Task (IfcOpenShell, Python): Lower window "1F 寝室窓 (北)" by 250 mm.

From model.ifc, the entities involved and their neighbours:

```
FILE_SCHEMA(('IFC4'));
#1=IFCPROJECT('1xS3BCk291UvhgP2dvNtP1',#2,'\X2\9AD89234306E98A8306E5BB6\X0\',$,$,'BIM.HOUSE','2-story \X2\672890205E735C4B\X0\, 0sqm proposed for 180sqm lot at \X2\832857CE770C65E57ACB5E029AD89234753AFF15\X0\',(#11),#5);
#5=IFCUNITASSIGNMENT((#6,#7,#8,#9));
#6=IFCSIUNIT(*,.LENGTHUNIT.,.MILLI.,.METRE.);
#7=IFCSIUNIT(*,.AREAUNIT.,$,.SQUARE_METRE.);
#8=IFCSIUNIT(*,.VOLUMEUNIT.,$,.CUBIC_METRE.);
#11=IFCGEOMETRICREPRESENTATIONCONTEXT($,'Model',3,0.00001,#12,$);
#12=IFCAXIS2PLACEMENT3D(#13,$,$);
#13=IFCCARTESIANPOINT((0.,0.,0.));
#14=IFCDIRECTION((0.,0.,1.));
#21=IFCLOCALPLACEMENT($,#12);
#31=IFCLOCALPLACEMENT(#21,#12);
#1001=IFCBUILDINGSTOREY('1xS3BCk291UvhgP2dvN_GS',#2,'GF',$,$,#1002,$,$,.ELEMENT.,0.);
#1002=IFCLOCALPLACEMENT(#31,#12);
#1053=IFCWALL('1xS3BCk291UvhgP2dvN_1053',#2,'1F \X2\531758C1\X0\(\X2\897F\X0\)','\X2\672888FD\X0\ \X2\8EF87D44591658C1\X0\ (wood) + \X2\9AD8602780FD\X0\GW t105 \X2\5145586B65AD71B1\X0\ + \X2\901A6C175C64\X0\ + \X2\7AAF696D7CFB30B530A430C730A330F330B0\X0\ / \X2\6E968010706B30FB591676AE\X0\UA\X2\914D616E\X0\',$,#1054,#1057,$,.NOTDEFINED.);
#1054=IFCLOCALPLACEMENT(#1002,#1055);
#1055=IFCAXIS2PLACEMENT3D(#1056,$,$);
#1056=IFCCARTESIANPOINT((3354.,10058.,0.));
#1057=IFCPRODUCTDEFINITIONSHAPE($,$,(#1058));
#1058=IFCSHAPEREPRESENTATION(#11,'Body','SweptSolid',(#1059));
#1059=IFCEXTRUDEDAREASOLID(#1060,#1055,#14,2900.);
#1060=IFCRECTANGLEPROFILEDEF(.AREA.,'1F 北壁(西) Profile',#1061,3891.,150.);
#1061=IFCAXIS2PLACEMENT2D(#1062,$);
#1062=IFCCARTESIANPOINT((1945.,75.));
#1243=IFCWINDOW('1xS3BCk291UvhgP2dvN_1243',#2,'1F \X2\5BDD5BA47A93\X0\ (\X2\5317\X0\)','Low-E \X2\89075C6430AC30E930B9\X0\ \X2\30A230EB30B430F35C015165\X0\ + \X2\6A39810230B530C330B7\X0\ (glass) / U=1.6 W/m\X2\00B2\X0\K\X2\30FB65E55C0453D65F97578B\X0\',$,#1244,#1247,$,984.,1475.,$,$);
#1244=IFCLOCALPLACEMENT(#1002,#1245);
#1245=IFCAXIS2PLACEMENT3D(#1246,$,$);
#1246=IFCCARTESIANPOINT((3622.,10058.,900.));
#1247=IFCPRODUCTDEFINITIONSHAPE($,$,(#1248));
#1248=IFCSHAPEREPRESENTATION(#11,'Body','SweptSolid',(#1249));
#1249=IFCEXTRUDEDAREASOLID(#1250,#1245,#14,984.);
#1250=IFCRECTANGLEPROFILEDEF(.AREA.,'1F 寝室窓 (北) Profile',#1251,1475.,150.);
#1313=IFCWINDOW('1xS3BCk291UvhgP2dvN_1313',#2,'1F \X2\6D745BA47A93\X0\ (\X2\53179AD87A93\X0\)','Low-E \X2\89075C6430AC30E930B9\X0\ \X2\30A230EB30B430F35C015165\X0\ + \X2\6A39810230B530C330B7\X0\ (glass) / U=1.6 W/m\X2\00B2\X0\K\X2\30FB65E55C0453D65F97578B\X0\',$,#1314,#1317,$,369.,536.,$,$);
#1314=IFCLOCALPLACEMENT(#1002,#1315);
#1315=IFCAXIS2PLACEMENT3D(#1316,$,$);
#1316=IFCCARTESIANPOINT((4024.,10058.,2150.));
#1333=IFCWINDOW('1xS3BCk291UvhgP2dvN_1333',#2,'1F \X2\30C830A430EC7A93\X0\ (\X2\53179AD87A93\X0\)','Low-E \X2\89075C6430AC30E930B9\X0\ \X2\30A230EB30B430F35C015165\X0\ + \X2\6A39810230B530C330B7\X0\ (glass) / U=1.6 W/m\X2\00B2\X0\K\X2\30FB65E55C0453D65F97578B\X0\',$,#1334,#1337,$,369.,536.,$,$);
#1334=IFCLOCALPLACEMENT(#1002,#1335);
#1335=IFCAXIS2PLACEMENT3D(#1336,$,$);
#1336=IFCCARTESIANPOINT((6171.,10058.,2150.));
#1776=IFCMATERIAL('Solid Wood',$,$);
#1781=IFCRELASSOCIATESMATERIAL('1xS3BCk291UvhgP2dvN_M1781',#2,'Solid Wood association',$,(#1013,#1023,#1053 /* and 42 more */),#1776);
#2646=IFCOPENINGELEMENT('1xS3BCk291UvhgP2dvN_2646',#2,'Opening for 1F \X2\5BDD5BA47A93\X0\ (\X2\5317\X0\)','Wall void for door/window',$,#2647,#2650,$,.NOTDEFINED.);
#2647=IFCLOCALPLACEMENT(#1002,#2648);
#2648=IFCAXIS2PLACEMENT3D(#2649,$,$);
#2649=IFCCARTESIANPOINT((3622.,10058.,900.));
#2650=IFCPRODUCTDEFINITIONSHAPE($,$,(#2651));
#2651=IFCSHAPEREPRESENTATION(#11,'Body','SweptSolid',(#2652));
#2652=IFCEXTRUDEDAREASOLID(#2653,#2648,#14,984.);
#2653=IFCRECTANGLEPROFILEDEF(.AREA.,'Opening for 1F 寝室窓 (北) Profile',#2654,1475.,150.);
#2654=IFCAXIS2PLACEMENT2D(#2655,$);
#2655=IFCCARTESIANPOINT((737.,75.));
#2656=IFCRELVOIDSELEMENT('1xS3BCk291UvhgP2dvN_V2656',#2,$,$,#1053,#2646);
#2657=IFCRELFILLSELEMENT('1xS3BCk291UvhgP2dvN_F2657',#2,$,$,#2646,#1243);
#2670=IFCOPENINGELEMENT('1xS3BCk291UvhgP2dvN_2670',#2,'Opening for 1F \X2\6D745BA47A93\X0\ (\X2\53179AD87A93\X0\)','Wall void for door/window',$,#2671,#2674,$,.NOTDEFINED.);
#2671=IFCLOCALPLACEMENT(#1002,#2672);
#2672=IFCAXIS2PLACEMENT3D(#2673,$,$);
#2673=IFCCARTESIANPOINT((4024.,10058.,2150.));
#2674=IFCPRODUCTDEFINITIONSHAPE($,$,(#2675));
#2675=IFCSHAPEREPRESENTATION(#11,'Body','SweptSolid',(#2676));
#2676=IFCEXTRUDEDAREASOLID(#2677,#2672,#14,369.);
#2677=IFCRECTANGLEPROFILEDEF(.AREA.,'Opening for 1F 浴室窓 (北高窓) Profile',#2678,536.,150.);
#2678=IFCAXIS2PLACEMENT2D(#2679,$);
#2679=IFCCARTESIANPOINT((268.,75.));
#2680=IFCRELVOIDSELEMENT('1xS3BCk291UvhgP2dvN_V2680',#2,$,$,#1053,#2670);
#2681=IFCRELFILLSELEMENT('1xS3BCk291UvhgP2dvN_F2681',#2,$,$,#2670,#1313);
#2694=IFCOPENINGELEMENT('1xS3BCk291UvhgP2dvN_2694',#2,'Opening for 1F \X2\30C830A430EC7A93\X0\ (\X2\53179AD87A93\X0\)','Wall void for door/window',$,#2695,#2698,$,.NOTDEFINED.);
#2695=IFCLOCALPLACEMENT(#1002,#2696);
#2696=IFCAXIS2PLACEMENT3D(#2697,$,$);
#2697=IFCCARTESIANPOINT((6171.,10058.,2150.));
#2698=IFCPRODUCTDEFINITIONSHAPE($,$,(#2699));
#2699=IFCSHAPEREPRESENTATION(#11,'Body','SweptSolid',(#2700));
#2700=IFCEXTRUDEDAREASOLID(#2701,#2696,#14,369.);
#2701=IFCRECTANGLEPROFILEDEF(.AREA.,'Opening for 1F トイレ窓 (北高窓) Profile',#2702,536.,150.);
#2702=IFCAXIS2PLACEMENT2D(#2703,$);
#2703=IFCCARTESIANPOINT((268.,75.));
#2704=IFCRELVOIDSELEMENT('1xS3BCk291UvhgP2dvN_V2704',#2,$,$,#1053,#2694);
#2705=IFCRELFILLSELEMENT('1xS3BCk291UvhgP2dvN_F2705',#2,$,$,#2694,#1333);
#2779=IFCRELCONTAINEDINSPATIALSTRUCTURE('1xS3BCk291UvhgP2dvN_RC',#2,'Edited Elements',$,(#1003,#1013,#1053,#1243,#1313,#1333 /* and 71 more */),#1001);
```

```python
import numpy as np
import ifcopenshell
import ifcopenshell.api.geometry
import ifcopenshell.util.placement
import ifcopenshell.util.unit

model = ifcopenshell.open("model.ifc")
unit_scale = ifcopenshell.util.unit.calculate_unit_scale(model)

window = model.by_guid("1xS3BCk291UvhgP2dvN_1243")
opening = window.FillsVoids[0].RelatingOpeningElement
dz = -0.25 / unit_scale

shift = np.array([0.0, 0.0, dz])
# The window is not placed relative to its opening, so move both.
for product in (opening, window):
    matrix = ifcopenshell.util.placement.get_local_placement(product.ObjectPlacement)
    matrix[:3, 3] += shift
    ifcopenshell.api.geometry.edit_object_placement(model, product=product, matrix=matrix, is_si=False)

print(f"moved by {dz * unit_scale:+.3f} m")

model.write("model_edited.ifc")
```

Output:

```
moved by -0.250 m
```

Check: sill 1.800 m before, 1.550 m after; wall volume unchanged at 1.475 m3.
